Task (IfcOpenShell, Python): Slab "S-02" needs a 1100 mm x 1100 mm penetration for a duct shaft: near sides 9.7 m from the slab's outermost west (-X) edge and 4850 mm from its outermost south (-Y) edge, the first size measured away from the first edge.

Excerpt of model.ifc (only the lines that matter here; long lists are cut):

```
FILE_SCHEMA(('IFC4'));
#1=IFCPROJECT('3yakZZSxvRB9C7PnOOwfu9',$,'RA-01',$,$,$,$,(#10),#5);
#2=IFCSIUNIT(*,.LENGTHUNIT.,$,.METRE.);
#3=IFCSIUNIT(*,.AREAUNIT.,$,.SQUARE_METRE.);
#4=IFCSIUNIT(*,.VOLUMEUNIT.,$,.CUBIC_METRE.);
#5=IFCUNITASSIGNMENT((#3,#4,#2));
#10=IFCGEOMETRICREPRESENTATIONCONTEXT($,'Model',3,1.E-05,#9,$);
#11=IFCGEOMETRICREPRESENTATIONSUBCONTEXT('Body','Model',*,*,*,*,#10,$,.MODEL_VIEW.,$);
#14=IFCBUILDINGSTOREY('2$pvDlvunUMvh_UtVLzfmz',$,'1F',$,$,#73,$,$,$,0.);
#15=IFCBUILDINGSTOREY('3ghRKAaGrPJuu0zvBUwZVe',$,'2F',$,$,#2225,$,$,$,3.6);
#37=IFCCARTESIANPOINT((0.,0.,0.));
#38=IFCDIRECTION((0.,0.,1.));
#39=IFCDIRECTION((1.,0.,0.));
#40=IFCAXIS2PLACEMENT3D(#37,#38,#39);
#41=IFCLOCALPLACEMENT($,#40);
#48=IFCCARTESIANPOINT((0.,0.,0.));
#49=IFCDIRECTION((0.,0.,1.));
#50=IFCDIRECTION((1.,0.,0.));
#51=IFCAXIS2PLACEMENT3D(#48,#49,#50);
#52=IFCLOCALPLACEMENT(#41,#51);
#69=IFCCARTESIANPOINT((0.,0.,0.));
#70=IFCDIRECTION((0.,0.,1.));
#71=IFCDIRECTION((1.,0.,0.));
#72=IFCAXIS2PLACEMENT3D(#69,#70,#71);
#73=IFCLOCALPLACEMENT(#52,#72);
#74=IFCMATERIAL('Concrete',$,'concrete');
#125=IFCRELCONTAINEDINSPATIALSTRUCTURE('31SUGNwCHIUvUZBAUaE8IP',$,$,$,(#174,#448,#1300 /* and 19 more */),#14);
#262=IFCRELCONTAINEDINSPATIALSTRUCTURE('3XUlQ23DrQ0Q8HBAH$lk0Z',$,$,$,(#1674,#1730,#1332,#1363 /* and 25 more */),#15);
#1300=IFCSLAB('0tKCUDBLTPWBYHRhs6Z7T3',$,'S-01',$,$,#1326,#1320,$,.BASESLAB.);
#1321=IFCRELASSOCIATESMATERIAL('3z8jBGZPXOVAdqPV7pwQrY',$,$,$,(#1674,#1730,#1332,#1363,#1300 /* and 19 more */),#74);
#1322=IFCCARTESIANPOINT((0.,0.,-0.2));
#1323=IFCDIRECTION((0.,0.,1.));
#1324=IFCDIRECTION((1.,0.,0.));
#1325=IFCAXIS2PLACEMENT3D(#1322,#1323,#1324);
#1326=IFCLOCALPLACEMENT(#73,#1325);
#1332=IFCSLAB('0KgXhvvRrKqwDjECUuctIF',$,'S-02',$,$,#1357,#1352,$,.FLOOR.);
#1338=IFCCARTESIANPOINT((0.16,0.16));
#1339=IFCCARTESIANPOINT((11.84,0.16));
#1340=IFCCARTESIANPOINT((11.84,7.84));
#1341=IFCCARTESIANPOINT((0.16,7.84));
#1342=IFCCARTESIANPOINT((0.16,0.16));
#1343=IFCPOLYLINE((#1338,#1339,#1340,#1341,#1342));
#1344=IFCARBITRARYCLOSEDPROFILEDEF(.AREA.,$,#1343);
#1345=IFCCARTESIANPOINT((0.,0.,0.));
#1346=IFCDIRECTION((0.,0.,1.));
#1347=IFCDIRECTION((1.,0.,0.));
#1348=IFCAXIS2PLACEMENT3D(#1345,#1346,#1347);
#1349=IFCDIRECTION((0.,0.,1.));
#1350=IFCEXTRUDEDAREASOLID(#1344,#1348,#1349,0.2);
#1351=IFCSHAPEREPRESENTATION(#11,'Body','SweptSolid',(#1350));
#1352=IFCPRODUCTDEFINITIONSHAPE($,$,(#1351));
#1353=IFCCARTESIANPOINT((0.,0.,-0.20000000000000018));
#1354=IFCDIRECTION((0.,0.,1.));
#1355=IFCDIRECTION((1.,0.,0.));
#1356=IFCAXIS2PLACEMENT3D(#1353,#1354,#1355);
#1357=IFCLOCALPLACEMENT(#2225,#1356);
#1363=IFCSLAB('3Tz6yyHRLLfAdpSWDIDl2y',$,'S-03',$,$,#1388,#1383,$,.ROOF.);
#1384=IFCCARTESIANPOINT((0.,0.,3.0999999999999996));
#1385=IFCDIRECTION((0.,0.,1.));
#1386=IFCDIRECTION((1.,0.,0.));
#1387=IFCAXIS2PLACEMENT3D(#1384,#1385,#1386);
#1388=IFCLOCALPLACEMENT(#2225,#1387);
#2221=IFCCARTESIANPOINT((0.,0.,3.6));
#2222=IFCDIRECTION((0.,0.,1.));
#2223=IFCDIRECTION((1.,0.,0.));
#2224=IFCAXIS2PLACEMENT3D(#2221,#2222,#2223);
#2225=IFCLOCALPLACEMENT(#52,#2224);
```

```python
import numpy as np
import ifcopenshell
import ifcopenshell.api.feature
import ifcopenshell.api.geometry
import ifcopenshell.api.root
import ifcopenshell.geom
import ifcopenshell.util.placement
import ifcopenshell.util.representation
import ifcopenshell.util.shape
import ifcopenshell.util.unit

model = ifcopenshell.open("model.ifc")
unit_scale = ifcopenshell.util.unit.calculate_unit_scale(model)
settings = ifcopenshell.geom.settings()


def volume(element):
    """Net volume in cubic metres, openings subtracted."""
    shape = ifcopenshell.geom.create_shape(settings, element)
    return ifcopenshell.util.shape.get_volume(shape.geometry)


slab = model.by_guid("0KgXhvvRrKqwDjECUuctIF")
before = volume(slab)

# Extent in the slab's own axes, in metres. The edges named are its -X and -Y sides.
slab_shape = ifcopenshell.geom.create_shape(settings, slab)
vertices = ifcopenshell.util.shape.get_vertices(slab_shape.geometry)
x_min, y_min, bottom = vertices.min(axis=0)
top = vertices[:, 2].max()

opening = ifcopenshell.api.root.create_entity(model, ifc_class="IfcOpeningElement", name="Duct shaft opening", predefined_type="OPENING")
context = ifcopenshell.util.representation.get_context(model, "Model", "Body", "MODEL_VIEW")
width, depth = 1.1, 1.1
outline = [(0.0, 0.0), (width, 0.0), (width, depth), (0.0, depth), (0.0, 0.0)]
# Overshoot both faces by 50 mm so the cut is clean.
shape = ifcopenshell.api.geometry.add_slab_representation(
    model, context=context, depth=top - bottom + 0.1, polyline=outline
)
ifcopenshell.api.geometry.assign_representation(model, product=opening, representation=shape)

matrix = ifcopenshell.util.placement.get_local_placement(slab.ObjectPlacement)
matrix[:, 3] = matrix @ np.append(np.array([x_min + 9.7, y_min + 4.85, bottom - 0.05]) / unit_scale, 1.0)
ifcopenshell.api.geometry.edit_object_placement(model, product=opening, matrix=matrix, is_si=False)
ifcopenshell.api.feature.add_feature(model, feature=opening, element=slab)

after = volume(slab)

print(f"slab volume {before:.3f} -> {after:.3f} m3")

model.write("model_edited.ifc")
```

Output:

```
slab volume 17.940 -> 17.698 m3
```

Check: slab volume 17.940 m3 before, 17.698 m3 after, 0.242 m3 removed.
